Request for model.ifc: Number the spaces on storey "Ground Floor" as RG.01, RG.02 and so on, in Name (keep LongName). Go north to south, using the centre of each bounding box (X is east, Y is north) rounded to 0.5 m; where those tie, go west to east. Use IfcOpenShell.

First a look at what the model holds.

```python
import ifcopenshell
import ifcopenshell.util.element
import ifcopenshell.util.placement

model = ifcopenshell.open("model.ifc")
print(model.schema)
storey = next(s for s in model.by_type("IfcBuildingStorey") if s.Name == "Ground Floor")
spaces = [e for e in ifcopenshell.util.element.get_decomposition(storey) if e.is_a("IfcSpace")]
for e in sorted(spaces, key=lambda e: e.id()):
    origin = ifcopenshell.util.placement.get_local_placement(e.ObjectPlacement)[:3, 3]
    print(e.id(), e.Name, e.LongName, origin.round(2) + 0.0, sep=" | ")
```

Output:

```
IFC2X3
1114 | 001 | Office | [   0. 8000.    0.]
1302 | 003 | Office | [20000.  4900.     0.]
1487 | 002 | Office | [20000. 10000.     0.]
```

```python
import ifcopenshell
import ifcopenshell.geom
import ifcopenshell.util.element
import ifcopenshell.util.shape

model = ifcopenshell.open("model.ifc")
settings = ifcopenshell.geom.settings()
settings.set("use-world-coords", True)


def centre(element):
    shape = ifcopenshell.geom.create_shape(settings, element)
    return ifcopenshell.util.shape.get_bbox_centroid(shape.geometry)


storey = next(s for s in model.by_type("IfcBuildingStorey") if s.Name == "Ground Floor")
spaces = [e for e in ifcopenshell.util.element.get_decomposition(storey) if e.is_a("IfcSpace")]

# Insertion points can sit at a corner or the storey origin, so sort by the geometry (in metres).
centres = {e: centre(e) for e in spaces}
spaces.sort(key=lambda e: (-round(centres[e][1] / 0.5), centres[e][0]))

for i, e in enumerate(spaces, start=1):
    number = f"RG.{i:02d}"
    e.Name = number
    print(e.id(), number)

model.write("model_v2.ifc")
```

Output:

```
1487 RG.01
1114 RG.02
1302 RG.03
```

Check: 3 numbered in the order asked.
